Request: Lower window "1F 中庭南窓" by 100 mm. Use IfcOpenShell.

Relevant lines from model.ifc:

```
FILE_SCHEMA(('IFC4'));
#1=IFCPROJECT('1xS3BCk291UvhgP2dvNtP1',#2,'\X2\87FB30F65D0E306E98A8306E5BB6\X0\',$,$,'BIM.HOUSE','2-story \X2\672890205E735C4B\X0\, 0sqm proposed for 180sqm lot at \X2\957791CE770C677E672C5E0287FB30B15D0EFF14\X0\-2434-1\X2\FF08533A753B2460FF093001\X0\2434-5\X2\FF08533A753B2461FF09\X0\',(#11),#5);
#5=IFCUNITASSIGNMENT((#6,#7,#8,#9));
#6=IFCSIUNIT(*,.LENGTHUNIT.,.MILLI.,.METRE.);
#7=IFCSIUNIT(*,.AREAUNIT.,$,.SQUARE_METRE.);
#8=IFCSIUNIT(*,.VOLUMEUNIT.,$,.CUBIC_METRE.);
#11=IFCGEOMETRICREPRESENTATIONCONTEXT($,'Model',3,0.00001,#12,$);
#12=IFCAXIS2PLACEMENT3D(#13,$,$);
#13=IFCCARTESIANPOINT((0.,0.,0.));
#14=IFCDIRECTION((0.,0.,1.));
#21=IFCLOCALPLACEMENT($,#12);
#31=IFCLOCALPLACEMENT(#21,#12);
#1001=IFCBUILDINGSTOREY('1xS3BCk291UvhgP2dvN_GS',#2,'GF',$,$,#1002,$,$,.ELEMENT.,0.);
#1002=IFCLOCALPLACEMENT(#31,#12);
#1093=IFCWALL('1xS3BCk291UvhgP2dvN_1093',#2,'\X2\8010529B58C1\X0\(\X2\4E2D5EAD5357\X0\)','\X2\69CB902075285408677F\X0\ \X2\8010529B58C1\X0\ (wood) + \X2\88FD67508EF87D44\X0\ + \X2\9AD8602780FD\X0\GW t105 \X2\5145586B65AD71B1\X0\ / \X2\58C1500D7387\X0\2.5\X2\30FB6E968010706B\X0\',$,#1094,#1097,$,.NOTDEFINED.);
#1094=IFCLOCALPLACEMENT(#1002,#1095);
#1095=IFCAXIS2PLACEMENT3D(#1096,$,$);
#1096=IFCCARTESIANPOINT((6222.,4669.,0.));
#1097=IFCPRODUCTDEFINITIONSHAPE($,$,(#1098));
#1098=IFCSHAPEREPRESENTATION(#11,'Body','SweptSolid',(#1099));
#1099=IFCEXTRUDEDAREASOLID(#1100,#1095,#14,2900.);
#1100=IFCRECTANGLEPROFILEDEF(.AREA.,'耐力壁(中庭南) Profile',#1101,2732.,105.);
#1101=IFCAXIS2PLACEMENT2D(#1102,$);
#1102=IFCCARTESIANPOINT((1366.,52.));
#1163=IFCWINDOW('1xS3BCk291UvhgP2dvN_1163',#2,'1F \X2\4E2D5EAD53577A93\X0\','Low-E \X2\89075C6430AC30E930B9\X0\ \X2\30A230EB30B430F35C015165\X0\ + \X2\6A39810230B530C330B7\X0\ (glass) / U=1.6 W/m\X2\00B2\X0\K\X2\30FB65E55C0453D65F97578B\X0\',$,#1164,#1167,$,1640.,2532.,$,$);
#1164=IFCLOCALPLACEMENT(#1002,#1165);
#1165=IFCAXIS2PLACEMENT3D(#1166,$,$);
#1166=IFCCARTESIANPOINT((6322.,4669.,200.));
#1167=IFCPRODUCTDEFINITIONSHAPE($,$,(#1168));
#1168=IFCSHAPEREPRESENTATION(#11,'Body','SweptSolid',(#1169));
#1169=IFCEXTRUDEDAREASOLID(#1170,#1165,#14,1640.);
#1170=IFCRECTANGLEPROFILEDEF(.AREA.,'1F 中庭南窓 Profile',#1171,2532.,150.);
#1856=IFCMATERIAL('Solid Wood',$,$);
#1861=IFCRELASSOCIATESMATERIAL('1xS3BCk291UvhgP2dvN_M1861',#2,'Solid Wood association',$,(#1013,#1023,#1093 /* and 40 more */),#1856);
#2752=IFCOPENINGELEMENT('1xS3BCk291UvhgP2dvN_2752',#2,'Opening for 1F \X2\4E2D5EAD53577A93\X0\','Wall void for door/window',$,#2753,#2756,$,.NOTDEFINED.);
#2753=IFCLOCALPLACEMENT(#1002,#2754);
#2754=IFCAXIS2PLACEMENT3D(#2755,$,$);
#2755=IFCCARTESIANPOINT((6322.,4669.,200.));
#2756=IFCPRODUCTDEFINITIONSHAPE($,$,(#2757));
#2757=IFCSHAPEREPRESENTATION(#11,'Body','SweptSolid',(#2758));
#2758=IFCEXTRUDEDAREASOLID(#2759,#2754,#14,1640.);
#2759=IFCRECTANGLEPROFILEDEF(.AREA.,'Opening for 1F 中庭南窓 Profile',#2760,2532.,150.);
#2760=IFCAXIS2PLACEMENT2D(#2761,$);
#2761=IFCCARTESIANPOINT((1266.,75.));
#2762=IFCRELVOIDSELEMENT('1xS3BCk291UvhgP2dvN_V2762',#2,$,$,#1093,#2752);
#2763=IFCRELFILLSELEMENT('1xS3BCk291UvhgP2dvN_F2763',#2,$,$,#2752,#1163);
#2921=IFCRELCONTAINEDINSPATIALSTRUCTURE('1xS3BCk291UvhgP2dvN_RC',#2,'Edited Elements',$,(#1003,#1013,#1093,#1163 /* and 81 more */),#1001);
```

```python
import numpy as np
import ifcopenshell
import ifcopenshell.api.geometry
import ifcopenshell.util.placement
import ifcopenshell.util.unit

model = ifcopenshell.open("model.ifc")
unit_scale = ifcopenshell.util.unit.calculate_unit_scale(model)

window = model.by_guid("1xS3BCk291UvhgP2dvN_1163")
opening = window.FillsVoids[0].RelatingOpeningElement
dz = -0.1 / unit_scale

shift = np.array([0.0, 0.0, dz])
# The window is not placed relative to its opening, so move both.
for product in (opening, window):
    matrix = ifcopenshell.util.placement.get_local_placement(product.ObjectPlacement)
    matrix[:3, 3] += shift
    ifcopenshell.api.geometry.edit_object_placement(model, product=product, matrix=matrix, is_si=False)

print(f"moved by {dz * unit_scale:+.3f} m")

model.write("model_v2.ifc")
```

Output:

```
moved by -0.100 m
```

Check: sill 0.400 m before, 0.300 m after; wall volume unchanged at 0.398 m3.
